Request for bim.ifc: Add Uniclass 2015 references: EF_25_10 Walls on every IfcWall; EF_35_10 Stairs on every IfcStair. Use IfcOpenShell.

First a look at what the model holds.

```python
import ifcopenshell

model = ifcopenshell.open("bim.ifc")
print(model.schema)
print("classifications:", [c.Name for c in model.by_type("IfcClassification")])
for ifc_class in ("IfcDoor", "IfcRoof", "IfcStair", "IfcWall", "IfcWindow"):
    print(ifc_class, len(model.by_type(ifc_class)))
```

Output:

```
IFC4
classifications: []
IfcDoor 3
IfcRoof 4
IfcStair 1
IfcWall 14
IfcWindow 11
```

```python
import ifcopenshell
import ifcopenshell.api.classification

model = ifcopenshell.open("bim.ifc")

system = ifcopenshell.api.classification.add_classification(model, classification="Uniclass 2015")

codes = {
    "IfcWall": ("EF_25_10", "Walls"),
    "IfcStair": ("EF_35_10", "Stairs"),
}
for ifc_class, (code, name) in codes.items():
    products = model.by_type(ifc_class)
    ifcopenshell.api.classification.add_reference(
        model, products=products, classification=system, identification=code, name=name
    )
    print(code, len(products))

model.write("bim-out.ifc")
```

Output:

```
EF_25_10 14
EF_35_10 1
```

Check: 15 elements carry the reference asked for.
